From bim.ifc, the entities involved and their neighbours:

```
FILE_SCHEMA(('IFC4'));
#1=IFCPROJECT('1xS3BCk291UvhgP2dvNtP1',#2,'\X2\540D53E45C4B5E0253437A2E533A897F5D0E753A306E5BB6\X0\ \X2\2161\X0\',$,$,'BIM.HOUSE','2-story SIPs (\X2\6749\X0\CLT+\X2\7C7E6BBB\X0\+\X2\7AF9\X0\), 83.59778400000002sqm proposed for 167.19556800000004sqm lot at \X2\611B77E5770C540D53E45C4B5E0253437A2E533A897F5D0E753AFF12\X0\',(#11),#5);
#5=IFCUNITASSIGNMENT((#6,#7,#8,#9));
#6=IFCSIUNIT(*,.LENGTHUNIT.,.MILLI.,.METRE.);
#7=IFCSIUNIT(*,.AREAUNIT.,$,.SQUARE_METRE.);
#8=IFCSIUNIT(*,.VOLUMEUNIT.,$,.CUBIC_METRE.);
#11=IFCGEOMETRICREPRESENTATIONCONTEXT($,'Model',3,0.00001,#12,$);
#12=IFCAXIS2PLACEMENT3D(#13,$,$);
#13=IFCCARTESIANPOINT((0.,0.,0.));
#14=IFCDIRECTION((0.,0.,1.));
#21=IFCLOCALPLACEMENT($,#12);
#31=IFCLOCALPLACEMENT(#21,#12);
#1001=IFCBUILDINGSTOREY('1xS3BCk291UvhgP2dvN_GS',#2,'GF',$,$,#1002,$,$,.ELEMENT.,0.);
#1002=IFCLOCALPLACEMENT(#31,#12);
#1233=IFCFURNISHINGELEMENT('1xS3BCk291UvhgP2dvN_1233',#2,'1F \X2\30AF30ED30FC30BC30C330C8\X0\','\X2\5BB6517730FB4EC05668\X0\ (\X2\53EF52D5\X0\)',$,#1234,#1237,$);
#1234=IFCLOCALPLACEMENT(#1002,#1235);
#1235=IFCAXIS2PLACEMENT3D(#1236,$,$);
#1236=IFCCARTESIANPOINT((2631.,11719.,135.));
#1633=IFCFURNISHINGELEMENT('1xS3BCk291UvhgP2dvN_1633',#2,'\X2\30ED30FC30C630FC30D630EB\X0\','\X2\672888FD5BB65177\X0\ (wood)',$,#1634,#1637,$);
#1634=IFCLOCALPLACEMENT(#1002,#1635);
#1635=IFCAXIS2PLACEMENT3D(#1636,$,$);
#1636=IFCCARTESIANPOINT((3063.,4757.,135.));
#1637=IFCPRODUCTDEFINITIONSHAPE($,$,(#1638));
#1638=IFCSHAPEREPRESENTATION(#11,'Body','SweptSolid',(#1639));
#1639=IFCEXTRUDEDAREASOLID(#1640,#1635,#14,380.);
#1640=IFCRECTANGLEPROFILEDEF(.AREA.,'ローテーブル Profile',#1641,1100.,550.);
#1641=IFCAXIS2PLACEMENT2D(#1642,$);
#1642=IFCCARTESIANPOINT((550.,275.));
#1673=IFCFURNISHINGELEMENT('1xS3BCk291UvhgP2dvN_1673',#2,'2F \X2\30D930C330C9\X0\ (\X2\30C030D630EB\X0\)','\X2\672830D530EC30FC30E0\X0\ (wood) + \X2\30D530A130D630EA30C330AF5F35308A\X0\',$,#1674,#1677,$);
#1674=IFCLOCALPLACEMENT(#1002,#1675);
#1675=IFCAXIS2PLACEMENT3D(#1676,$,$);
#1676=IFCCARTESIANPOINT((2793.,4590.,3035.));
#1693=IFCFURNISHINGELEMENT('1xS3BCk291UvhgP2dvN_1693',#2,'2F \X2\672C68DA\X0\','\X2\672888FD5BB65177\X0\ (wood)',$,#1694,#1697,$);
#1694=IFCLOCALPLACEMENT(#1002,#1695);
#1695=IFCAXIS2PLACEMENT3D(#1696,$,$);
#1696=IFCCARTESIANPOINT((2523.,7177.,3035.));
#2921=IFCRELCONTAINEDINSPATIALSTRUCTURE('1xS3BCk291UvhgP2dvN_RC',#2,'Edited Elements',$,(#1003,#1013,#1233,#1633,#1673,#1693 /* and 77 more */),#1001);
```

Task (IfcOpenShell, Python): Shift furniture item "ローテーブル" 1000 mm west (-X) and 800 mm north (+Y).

```python
import ifcopenshell
import ifcopenshell.api.geometry
import ifcopenshell.util.placement

model = ifcopenshell.open("bim.ifc")

item = model.by_id(1633)
matrix = ifcopenshell.util.placement.get_local_placement(item.ObjectPlacement)
matrix[0, 3] -= 1000.0
matrix[1, 3] += 800.0
ifcopenshell.api.geometry.edit_object_placement(model, product=item, matrix=matrix, is_si=False)

print(ifcopenshell.util.placement.get_local_placement(item.ObjectPlacement).round(3) + 0.0)

model.write("bim-out.ifc")
```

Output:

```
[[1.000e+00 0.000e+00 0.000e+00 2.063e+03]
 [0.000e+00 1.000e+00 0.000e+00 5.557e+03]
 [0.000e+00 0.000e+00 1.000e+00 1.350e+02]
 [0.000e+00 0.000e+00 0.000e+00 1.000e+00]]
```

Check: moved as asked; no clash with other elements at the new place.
